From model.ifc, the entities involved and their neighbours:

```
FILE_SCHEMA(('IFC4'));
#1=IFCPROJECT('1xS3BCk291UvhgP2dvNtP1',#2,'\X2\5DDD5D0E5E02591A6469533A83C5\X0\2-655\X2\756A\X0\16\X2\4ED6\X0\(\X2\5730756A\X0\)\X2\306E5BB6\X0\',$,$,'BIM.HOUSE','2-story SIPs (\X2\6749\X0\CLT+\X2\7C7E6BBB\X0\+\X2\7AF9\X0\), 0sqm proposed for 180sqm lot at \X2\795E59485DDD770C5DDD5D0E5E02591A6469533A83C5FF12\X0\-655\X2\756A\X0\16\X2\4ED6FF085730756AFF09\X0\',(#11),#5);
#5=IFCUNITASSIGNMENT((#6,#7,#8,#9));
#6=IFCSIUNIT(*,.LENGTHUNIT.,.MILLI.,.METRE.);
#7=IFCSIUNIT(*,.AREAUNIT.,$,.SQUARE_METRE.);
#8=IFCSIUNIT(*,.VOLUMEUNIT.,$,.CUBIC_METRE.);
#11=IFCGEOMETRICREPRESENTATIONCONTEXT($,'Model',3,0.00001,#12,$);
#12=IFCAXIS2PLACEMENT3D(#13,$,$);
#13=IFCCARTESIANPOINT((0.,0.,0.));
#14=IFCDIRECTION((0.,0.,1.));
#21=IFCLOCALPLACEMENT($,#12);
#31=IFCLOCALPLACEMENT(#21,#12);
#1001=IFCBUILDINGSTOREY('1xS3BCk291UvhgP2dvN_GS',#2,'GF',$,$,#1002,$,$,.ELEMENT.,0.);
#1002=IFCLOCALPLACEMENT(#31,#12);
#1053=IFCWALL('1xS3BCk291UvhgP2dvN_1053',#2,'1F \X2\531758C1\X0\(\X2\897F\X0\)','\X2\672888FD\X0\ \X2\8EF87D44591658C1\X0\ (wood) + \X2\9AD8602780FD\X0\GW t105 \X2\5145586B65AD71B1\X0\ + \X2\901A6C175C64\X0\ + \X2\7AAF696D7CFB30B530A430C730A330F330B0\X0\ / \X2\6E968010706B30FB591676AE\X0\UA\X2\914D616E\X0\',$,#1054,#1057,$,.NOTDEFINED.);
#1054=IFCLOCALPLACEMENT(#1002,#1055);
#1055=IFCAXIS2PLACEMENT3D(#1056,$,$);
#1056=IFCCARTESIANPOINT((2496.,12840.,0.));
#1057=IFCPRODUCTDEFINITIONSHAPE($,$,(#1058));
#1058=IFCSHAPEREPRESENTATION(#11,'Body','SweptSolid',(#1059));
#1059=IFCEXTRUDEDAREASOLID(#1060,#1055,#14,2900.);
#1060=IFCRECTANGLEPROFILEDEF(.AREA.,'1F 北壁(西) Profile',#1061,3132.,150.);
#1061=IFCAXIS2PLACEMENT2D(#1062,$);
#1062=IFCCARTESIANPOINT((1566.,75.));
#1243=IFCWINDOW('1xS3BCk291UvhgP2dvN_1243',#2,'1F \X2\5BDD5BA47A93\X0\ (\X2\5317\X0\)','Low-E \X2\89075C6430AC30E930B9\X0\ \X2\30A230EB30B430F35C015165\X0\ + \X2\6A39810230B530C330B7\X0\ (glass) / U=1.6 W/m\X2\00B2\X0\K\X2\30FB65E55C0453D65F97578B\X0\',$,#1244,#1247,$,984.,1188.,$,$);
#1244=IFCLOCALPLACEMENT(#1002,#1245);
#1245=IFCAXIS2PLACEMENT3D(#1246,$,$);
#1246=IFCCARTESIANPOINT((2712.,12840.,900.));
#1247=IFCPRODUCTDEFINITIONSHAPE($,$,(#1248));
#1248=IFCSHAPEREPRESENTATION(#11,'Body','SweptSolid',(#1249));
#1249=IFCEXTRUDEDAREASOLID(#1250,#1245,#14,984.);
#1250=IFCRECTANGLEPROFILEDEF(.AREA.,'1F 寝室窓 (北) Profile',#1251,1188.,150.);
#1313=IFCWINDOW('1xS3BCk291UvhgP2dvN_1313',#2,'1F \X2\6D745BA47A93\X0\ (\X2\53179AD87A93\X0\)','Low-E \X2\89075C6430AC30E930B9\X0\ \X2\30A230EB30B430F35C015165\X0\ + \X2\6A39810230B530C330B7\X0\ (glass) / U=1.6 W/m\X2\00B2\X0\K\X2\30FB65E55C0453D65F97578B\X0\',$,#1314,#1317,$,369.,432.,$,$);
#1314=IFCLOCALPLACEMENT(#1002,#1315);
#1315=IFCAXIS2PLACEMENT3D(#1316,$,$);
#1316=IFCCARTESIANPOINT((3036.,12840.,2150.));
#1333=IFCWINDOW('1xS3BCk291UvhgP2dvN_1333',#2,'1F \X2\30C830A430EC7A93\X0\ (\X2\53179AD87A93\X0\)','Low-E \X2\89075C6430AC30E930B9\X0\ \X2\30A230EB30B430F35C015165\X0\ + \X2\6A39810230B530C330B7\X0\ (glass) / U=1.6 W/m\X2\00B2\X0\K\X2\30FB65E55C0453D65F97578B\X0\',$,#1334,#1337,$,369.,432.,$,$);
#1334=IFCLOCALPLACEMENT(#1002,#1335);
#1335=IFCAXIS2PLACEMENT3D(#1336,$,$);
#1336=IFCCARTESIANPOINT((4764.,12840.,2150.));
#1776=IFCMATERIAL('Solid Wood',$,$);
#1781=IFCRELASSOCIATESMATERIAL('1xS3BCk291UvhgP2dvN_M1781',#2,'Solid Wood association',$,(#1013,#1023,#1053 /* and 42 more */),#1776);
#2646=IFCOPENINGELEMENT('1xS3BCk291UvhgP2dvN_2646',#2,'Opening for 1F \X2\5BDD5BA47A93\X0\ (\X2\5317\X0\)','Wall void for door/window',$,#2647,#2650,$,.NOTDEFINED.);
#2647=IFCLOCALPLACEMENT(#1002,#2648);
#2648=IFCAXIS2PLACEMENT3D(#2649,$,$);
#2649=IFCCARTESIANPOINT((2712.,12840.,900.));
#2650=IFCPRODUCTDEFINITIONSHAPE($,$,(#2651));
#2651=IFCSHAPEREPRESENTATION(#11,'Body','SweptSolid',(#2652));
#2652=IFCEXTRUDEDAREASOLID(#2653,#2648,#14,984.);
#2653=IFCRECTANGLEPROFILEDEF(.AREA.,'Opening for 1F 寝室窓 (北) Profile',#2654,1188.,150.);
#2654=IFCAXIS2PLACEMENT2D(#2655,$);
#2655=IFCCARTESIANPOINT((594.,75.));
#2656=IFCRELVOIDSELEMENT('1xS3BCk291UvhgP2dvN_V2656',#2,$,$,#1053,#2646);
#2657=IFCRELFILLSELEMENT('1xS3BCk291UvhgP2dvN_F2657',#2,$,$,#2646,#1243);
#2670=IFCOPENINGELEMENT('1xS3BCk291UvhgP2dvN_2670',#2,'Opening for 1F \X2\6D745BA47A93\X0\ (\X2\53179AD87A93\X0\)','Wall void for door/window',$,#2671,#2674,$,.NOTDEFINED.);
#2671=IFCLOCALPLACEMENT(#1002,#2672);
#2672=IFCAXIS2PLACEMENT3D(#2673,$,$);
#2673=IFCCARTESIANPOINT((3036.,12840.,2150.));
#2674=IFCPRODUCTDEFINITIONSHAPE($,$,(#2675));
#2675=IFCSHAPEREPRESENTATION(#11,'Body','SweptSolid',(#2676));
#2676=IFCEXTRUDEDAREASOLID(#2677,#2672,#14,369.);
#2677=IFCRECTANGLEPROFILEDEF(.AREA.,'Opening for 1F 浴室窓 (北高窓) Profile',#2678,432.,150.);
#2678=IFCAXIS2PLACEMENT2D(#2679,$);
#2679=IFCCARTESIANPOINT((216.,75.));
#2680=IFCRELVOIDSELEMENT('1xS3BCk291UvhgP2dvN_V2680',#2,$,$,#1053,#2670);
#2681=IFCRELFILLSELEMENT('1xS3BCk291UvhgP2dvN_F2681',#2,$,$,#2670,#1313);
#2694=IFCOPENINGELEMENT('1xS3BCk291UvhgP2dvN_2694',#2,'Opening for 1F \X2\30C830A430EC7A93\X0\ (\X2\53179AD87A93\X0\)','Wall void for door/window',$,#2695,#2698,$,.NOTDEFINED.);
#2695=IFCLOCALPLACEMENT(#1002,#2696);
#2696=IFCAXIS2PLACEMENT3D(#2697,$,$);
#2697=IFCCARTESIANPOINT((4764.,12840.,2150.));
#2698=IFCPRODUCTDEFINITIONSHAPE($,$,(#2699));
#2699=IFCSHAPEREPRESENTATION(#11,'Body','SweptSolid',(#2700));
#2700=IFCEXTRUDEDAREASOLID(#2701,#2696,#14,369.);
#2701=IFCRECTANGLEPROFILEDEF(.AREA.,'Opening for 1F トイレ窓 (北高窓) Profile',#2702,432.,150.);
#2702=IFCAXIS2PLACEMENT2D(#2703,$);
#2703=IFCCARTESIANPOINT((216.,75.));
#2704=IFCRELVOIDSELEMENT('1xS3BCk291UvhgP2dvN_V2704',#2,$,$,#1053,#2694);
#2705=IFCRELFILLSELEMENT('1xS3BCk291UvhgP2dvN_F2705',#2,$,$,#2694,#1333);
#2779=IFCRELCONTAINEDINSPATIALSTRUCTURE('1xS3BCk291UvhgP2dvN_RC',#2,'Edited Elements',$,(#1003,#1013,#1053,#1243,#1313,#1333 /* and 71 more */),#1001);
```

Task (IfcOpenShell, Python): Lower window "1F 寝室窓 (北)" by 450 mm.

```python
import numpy as np
import ifcopenshell
import ifcopenshell.api.geometry
import ifcopenshell.util.placement
import ifcopenshell.util.unit

model = ifcopenshell.open("model.ifc")
unit_scale = ifcopenshell.util.unit.calculate_unit_scale(model)

window = model.by_guid("1xS3BCk291UvhgP2dvN_1243")
opening = window.FillsVoids[0].RelatingOpeningElement
dz = -0.45 / unit_scale

shift = np.array([0.0, 0.0, dz])
# The window is not placed relative to its opening, so move both.
for product in (opening, window):
    matrix = ifcopenshell.util.placement.get_local_placement(product.ObjectPlacement)
    matrix[:3, 3] += shift
    ifcopenshell.api.geometry.edit_object_placement(model, product=product, matrix=matrix, is_si=False)

print(f"moved by {dz * unit_scale:+.3f} m")

model.write("model_edited.ifc")
```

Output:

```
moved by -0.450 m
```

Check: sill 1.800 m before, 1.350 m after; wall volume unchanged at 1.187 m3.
